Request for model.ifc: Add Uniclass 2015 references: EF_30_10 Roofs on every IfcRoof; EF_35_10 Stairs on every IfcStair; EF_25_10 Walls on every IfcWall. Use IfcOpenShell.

First a look at what the model holds.

```python
import ifcopenshell

model = ifcopenshell.open("model.ifc")
print(model.schema)
print("classifications:", [c.Name for c in model.by_type("IfcClassification")])
for ifc_class in ("IfcDoor", "IfcRoof", "IfcStair", "IfcWall", "IfcWindow"):
    print(ifc_class, len(model.by_type(ifc_class)))
```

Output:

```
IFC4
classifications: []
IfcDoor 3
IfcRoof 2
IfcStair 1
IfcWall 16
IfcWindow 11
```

```python
import ifcopenshell
import ifcopenshell.api.classification

model = ifcopenshell.open("model.ifc")

system = ifcopenshell.api.classification.add_classification(model, classification="Uniclass 2015")

codes = {
    "IfcRoof": ("EF_30_10", "Roofs"),
    "IfcStair": ("EF_35_10", "Stairs"),
    "IfcWall": ("EF_25_10", "Walls"),
}
for ifc_class, (code, name) in codes.items():
    products = model.by_type(ifc_class)
    ifcopenshell.api.classification.add_reference(
        model, products=products, classification=system, identification=code, name=name
    )
    print(code, len(products))

model.write("model_v2.ifc")
```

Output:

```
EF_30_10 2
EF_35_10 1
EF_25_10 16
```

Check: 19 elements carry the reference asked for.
